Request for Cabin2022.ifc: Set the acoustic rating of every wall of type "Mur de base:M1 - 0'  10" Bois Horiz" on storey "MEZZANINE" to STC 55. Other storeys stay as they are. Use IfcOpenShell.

First a look at what the model holds.

```python
import ifcopenshell
import ifcopenshell.util.element

model = ifcopenshell.open("Cabin2022.ifc")
print(model.schema)
storey = next(s for s in model.by_type("IfcBuildingStorey") if s.Name == "MEZZANINE")
walls = [e for e in ifcopenshell.util.element.get_decomposition(storey) if e.is_a("IfcWall")]
seen = {}
for e in walls:
    element_type = ifcopenshell.util.element.get_type(e)
    key = (element_type.Name if element_type != e and element_type else None, ifcopenshell.util.element.get_pset(e, "Pset_WallCommon", "AcousticRating"))
    seen[key] = seen.get(key, 0) + 1
for (name, value), count in sorted(seen.items(), key=str):
    print(count, "x", name, "|", value)
```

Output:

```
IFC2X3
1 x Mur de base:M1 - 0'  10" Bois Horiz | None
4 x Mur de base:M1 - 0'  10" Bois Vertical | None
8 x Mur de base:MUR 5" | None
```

```python
import ifcopenshell
import ifcopenshell.api.pset
import ifcopenshell.util.element

model = ifcopenshell.open("Cabin2022.ifc")

storey = next(s for s in model.by_type("IfcBuildingStorey") if s.Name == "MEZZANINE")
walls = [e for e in ifcopenshell.util.element.get_decomposition(storey) if e.is_a("IfcWall")]

count = 0
for e in walls:
    element_type = ifcopenshell.util.element.get_type(e)
    if element_type in (None, e) or element_type.Name != 'Mur de base:M1 - 0\'  10" Bois Horiz':
        continue
    # add_pset returns the element's existing set when there is one.
    pset = ifcopenshell.api.pset.add_pset(model, product=e, name="Pset_WallCommon")
    ifcopenshell.api.pset.edit_pset(model, pset=pset, properties={"AcousticRating": "STC 55"})
    count += 1

print(count, "walls updated")

model.write("Cabin2022-out.ifc")
```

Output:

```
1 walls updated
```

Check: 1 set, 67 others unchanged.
